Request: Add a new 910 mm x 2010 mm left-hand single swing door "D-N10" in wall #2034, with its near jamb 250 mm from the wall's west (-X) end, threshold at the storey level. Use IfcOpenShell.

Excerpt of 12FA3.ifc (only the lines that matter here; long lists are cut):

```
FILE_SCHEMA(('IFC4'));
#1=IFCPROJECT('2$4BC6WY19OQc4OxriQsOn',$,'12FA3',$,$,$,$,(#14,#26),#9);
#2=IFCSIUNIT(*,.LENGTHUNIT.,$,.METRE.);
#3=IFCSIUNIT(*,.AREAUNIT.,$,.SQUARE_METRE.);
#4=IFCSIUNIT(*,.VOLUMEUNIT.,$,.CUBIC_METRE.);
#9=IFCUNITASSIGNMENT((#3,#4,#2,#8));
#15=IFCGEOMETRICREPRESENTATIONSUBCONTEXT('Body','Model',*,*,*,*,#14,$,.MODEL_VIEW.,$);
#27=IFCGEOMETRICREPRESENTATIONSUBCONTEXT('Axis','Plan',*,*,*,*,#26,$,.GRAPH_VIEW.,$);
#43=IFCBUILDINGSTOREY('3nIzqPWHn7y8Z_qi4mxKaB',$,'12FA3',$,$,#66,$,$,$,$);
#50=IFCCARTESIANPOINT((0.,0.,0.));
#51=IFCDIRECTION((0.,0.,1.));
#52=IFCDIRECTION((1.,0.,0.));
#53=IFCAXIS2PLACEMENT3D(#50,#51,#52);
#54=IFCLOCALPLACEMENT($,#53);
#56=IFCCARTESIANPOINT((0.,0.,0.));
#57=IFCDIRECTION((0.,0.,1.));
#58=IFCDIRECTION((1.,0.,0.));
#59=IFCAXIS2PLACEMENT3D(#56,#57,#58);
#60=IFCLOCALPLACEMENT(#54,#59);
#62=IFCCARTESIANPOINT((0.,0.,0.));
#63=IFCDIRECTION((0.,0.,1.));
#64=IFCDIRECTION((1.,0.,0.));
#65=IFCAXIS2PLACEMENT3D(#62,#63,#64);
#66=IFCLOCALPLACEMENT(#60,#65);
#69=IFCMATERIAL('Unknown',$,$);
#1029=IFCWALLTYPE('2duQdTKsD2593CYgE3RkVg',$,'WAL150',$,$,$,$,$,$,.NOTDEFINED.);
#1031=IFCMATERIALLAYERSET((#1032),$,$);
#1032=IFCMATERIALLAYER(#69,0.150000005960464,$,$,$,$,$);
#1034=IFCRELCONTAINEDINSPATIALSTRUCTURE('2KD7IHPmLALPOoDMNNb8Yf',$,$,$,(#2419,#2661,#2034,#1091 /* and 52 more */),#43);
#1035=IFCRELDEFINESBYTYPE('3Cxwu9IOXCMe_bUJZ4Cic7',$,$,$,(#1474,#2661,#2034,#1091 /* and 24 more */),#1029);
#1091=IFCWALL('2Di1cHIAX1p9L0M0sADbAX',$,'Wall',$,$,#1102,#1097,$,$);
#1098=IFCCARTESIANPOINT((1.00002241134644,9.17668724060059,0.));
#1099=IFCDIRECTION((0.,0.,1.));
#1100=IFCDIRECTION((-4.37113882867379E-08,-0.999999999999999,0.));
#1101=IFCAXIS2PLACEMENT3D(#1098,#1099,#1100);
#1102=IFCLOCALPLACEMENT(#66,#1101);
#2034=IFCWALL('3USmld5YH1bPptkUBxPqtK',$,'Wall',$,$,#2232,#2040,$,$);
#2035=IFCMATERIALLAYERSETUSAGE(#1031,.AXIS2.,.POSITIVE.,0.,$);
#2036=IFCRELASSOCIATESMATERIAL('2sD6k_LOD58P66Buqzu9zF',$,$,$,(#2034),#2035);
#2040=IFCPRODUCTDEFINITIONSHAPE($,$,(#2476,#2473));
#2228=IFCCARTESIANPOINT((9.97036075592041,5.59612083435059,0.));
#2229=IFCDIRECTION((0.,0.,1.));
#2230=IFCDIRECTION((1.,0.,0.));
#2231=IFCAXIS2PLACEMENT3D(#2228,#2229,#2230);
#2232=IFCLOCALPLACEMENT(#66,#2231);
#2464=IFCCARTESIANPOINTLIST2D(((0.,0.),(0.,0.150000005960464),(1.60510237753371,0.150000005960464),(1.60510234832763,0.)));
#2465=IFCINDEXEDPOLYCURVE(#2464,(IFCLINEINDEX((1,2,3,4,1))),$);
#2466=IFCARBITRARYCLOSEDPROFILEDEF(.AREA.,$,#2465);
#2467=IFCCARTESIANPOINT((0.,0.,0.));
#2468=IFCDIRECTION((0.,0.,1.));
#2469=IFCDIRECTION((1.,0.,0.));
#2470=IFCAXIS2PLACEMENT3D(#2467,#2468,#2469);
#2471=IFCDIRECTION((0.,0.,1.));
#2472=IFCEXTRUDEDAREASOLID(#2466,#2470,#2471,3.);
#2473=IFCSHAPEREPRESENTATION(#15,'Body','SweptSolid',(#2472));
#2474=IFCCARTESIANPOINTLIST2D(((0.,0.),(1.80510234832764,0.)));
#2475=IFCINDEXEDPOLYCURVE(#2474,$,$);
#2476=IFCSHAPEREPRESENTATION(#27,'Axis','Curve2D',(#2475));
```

```python
import numpy as np
import ifcopenshell
import ifcopenshell.api.feature
import ifcopenshell.api.geometry
import ifcopenshell.api.root
import ifcopenshell.api.spatial
import ifcopenshell.geom
import ifcopenshell.util.element
import ifcopenshell.util.placement
import ifcopenshell.util.representation
import ifcopenshell.util.shape
import ifcopenshell.util.unit

model = ifcopenshell.open("12FA3.ifc")
unit_scale = ifcopenshell.util.unit.calculate_unit_scale(model)
settings = ifcopenshell.geom.settings()


def volume(element):
    """Net volume in cubic metres, openings subtracted."""
    shape = ifcopenshell.geom.create_shape(settings, element)
    return ifcopenshell.util.shape.get_volume(shape.geometry)


wall = model.by_id(2034)
storey = ifcopenshell.util.element.get_container(wall, ifc_class="IfcBuildingStorey")
context = ifcopenshell.util.representation.get_context(model, "Model", "Body", "MODEL_VIEW")
before = volume(wall)

width, height, from_end, sill = 0.91, 2.01, 0.25, 0.0  # metres

# The wall runs along its own X axis, and the end named is its -X end.
wall_shape = ifcopenshell.geom.create_shape(settings, wall)
x, y, z = ifcopenshell.util.shape.get_vertices(wall_shape.geometry).T
start = x.min() + from_end
face, thickness = float(y.min()), float(y.max() - y.min())
wall_matrix = ifcopenshell.util.placement.get_local_placement(wall.ObjectPlacement)
level = ifcopenshell.util.placement.get_local_placement(storey.ObjectPlacement)[2, 3]


def in_wall(x, y):
    """Placement at x, y metres in the wall's axes, at sill height."""
    matrix = wall_matrix.copy()
    matrix[:, 3] = wall_matrix @ np.array([x / unit_scale, y / unit_scale, 0.0, 1.0])
    matrix[2, 3] = level + sill / unit_scale
    return matrix


# Opening: a box that overshoots both wall faces by 50 mm.
opening = ifcopenshell.api.root.create_entity(model, ifc_class="IfcOpeningElement", predefined_type="OPENING")
box = ifcopenshell.api.geometry.add_wall_representation(
    model, context=context, length=width, height=height, thickness=thickness + 0.1
)
ifcopenshell.api.geometry.assign_representation(model, product=opening, representation=box)
ifcopenshell.api.geometry.edit_object_placement(model, product=opening, matrix=in_wall(start, face - 0.05), is_si=False)
ifcopenshell.api.feature.add_feature(model, feature=opening, element=wall)

door = ifcopenshell.api.root.create_entity(model, ifc_class="IfcDoor", name="D-N10", predefined_type="DOOR")
door.OverallWidth, door.OverallHeight = width / unit_scale, height / unit_scale
door.OperationType = "SINGLE_SWING_LEFT"
body = ifcopenshell.api.geometry.add_door_representation(
    model,
    context=context,
    overall_width=door.OverallWidth,
    overall_height=door.OverallHeight,
    operation_type="SINGLE_SWING_LEFT",
    lining_properties={"LiningDepth": thickness / unit_scale, "ThresholdDepth": thickness / unit_scale},
)
ifcopenshell.api.geometry.assign_representation(model, product=door, representation=body)
ifcopenshell.api.spatial.assign_container(model, products=[door], relating_structure=storey)
ifcopenshell.api.feature.add_filling(model, opening=opening, element=door)

# The lining spans the wall, so the door starts at the wall face.
ifcopenshell.api.geometry.edit_object_placement(model, product=door, matrix=in_wall(start, face), is_si=False)

after = volume(wall)

print(f"wall volume {before:.3f} -> {after:.3f} m3")

model.write("12FA3_rev.ifc")
```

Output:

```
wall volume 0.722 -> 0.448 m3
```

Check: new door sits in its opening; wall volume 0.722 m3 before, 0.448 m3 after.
